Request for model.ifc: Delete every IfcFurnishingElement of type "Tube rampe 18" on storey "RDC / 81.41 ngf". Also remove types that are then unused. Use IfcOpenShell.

First a look at what the model holds.

```python
import ifcopenshell
import ifcopenshell.util.element

model = ifcopenshell.open("model.ifc")
print(model.schema)
storey = next(s for s in model.by_type("IfcBuildingStorey") if s.Name == "RDC / 81.41 ngf")
furniture = [e for e in ifcopenshell.util.element.get_decomposition(storey) if e.is_a("IfcFurnishingElement")]
seen = {}
for e in furniture:
    element_type = ifcopenshell.util.element.get_type(e)
    name = element_type.Name if element_type not in (None, e) else None
    seen[name] = seen.get(name, 0) + 1
for name, count in sorted(seen.items(), key=str):
    print(count, "x", name)
```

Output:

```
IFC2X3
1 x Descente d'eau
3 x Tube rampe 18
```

```python
import ifcopenshell
import ifcopenshell.api.root
import ifcopenshell.util.element

model = ifcopenshell.open("model.ifc")

storey = next(s for s in model.by_type("IfcBuildingStorey") if s.Name == "RDC / 81.41 ngf")
furniture = [e for e in ifcopenshell.util.element.get_decomposition(storey) if e.is_a("IfcFurnishingElement")]
targets = [e for e in furniture if (t := ifcopenshell.util.element.get_type(e)) not in (None, e) and t.Name == "Tube rampe 18"]
types = {ifcopenshell.util.element.get_type(e) for e in targets} - {None, *targets}

for e in targets:
    ifcopenshell.api.root.remove_product(model, product=e)
print(len(targets), "removed")

unused = [t for t in types if not ifcopenshell.util.element.get_types(t)]
for t in unused:
    ifcopenshell.api.root.remove_product(model, product=t)
print(len(unused), "unused types removed")

model.write("model_rev.ifc")
```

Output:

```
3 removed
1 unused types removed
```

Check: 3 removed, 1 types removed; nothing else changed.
